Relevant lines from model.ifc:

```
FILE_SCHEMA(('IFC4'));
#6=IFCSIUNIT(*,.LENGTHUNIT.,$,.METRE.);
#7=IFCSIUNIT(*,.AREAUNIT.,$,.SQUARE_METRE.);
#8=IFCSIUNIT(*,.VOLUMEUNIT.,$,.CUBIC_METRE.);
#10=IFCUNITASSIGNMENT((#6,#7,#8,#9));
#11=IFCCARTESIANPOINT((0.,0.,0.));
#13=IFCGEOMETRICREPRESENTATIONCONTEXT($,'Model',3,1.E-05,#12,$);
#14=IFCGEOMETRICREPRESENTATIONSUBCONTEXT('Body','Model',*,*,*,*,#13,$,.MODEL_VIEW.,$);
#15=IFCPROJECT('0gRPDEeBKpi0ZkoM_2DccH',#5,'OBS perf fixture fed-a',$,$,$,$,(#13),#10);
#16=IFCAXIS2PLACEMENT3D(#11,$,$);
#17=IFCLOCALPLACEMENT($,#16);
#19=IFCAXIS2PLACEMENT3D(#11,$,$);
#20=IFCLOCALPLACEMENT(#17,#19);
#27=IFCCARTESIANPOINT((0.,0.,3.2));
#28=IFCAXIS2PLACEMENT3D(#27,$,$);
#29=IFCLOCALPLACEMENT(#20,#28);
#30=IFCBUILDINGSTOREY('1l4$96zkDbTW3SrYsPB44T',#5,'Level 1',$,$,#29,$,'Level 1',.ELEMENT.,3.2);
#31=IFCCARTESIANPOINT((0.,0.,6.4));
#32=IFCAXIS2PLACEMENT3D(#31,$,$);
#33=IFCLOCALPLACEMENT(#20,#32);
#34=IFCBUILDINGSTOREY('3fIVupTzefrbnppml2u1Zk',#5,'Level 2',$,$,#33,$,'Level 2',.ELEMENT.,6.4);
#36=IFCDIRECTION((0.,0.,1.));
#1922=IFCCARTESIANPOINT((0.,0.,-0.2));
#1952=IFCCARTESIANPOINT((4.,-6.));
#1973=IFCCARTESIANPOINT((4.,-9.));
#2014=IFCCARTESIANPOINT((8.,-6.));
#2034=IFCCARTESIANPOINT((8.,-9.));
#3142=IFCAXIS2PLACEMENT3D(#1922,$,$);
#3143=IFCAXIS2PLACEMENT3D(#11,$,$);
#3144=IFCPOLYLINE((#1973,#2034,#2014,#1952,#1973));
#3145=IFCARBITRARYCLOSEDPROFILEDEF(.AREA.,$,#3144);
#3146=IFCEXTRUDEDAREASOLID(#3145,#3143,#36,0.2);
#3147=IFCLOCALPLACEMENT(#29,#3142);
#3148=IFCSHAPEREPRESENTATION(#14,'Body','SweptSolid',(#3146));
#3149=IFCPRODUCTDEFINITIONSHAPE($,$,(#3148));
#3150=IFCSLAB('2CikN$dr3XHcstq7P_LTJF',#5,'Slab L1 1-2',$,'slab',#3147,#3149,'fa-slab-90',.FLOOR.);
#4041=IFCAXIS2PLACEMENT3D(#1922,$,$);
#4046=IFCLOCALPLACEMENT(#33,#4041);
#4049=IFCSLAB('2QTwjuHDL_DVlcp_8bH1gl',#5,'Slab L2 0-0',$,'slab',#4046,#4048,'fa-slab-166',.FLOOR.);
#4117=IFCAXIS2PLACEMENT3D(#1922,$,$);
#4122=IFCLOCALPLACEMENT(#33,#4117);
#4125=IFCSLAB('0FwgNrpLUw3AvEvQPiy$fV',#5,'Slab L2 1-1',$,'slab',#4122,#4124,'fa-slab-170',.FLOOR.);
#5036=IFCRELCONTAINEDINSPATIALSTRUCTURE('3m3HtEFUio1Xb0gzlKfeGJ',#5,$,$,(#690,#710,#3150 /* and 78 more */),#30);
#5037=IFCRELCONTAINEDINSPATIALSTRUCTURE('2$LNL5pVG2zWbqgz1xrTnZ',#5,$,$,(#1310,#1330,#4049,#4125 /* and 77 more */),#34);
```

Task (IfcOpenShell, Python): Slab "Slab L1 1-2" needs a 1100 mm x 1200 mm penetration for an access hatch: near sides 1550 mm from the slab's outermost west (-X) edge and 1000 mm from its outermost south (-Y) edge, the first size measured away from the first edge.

```python
import numpy as np
import ifcopenshell
import ifcopenshell.api.feature
import ifcopenshell.api.geometry
import ifcopenshell.api.root
import ifcopenshell.geom
import ifcopenshell.util.placement
import ifcopenshell.util.representation
import ifcopenshell.util.shape
import ifcopenshell.util.unit

model = ifcopenshell.open("model.ifc")
unit_scale = ifcopenshell.util.unit.calculate_unit_scale(model)
settings = ifcopenshell.geom.settings()


def volume(element):
    """Net volume in cubic metres, openings subtracted."""
    shape = ifcopenshell.geom.create_shape(settings, element)
    return ifcopenshell.util.shape.get_volume(shape.geometry)


slab = model.by_guid("2CikN$dr3XHcstq7P_LTJF")
before = volume(slab)

# Extent in the slab's own axes, in metres. The edges named are its -X and -Y sides.
slab_shape = ifcopenshell.geom.create_shape(settings, slab)
vertices = ifcopenshell.util.shape.get_vertices(slab_shape.geometry)
x_min, y_min, bottom = vertices.min(axis=0)
top = vertices[:, 2].max()

opening = ifcopenshell.api.root.create_entity(model, ifc_class="IfcOpeningElement", name="Access hatch opening", predefined_type="OPENING")
context = ifcopenshell.util.representation.get_context(model, "Model", "Body", "MODEL_VIEW")
width, depth = 1.1, 1.2
outline = [(0.0, 0.0), (width, 0.0), (width, depth), (0.0, depth), (0.0, 0.0)]
# Overshoot both faces by 50 mm so the cut is clean.
shape = ifcopenshell.api.geometry.add_slab_representation(
    model, context=context, depth=top - bottom + 0.1, polyline=outline
)
ifcopenshell.api.geometry.assign_representation(model, product=opening, representation=shape)

matrix = ifcopenshell.util.placement.get_local_placement(slab.ObjectPlacement)
matrix[:, 3] = matrix @ np.append(np.array([x_min + 1.55, y_min + 1, bottom - 0.05]) / unit_scale, 1.0)
ifcopenshell.api.geometry.edit_object_placement(model, product=opening, matrix=matrix, is_si=False)
ifcopenshell.api.feature.add_feature(model, feature=opening, element=slab)

after = volume(slab)

print(f"slab volume {before:.3f} -> {after:.3f} m3")

model.write("model_updated.ifc")
```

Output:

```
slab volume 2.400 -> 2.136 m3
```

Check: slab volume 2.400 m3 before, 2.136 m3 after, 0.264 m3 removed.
